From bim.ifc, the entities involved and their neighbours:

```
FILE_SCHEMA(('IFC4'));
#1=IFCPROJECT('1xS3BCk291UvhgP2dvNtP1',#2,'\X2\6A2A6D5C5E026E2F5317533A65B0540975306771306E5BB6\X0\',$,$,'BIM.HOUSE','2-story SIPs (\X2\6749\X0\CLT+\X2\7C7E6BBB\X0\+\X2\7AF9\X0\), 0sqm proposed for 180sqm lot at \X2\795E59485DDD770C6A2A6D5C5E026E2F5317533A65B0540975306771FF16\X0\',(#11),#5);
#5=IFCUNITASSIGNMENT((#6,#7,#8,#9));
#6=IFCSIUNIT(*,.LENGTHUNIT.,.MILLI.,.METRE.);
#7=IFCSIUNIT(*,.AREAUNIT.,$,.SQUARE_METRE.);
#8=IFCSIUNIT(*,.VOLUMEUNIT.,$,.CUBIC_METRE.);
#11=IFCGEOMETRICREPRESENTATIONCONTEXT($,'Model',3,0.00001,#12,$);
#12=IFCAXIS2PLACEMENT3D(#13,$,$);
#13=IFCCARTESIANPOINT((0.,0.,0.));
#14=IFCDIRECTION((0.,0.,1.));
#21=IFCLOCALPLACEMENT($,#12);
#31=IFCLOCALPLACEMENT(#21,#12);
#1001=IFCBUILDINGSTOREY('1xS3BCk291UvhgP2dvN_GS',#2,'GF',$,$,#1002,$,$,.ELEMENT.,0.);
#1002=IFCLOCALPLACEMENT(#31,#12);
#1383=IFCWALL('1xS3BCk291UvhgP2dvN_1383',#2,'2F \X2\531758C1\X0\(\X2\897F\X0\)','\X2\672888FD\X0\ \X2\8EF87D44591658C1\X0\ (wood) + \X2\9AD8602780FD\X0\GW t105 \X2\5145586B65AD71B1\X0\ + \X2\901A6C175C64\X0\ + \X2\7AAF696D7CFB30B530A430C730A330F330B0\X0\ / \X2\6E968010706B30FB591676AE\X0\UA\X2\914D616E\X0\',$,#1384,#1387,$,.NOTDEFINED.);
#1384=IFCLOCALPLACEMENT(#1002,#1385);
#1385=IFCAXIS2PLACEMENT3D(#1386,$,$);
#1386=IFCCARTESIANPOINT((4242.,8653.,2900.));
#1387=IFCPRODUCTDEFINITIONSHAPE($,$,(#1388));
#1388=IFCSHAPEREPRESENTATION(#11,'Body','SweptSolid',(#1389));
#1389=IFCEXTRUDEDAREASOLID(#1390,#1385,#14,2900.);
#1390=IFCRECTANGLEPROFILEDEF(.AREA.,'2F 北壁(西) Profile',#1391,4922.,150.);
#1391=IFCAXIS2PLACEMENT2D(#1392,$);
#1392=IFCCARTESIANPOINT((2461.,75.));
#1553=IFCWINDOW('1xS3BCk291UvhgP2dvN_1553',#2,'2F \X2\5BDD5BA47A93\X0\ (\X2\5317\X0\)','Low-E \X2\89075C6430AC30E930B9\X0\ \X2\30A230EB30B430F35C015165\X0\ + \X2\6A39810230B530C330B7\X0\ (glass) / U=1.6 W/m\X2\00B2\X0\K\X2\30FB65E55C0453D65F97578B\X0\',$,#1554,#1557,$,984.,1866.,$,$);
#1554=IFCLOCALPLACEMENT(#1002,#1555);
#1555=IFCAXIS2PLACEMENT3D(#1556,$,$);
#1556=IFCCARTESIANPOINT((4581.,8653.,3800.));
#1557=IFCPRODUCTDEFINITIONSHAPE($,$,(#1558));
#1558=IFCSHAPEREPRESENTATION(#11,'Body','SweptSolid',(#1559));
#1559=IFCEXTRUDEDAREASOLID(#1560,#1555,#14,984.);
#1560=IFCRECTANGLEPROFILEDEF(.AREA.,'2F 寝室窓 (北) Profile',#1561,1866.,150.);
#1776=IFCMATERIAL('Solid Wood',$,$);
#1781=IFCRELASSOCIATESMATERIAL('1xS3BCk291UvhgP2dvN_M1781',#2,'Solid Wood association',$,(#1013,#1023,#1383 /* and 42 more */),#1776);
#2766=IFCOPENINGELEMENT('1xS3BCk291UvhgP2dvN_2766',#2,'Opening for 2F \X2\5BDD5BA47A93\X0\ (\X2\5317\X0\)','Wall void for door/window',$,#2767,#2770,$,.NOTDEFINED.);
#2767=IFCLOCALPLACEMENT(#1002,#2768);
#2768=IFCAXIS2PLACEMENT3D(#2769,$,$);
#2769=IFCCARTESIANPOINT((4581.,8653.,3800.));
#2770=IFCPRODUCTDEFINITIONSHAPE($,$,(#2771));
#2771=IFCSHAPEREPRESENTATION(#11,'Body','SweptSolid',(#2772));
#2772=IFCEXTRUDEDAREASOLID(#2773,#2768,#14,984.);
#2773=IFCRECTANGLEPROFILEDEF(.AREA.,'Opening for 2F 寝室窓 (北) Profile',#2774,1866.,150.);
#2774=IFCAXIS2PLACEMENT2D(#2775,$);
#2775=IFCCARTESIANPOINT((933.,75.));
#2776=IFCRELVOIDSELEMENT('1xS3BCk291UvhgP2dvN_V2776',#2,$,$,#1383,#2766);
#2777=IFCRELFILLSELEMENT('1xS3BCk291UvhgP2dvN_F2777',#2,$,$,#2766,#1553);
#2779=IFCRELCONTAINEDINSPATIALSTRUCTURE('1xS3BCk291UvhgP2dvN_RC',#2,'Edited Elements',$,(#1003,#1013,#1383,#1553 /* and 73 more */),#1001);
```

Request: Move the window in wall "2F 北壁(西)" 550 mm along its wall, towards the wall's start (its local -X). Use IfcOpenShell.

```python
import ifcopenshell
import ifcopenshell.api.geometry
import ifcopenshell.util.placement

model = ifcopenshell.open("bim.ifc")

window = model.by_guid("1xS3BCk291UvhgP2dvN_1553")
opening = window.FillsVoids[0].RelatingOpeningElement
wall = opening.VoidsElements[0].RelatingBuildingElement

wall_matrix = ifcopenshell.util.placement.get_local_placement(wall.ObjectPlacement)
shift = wall_matrix[:3, 0] * -550.0
before = ifcopenshell.util.placement.get_local_placement(window.ObjectPlacement)[:3, 3].copy()

# The window is not placed relative to its opening, so move both.
for product in (opening, window):
    matrix = ifcopenshell.util.placement.get_local_placement(product.ObjectPlacement)
    matrix[:3, 3] += shift
    ifcopenshell.api.geometry.edit_object_placement(model, product=product, matrix=matrix, is_si=False)

after = ifcopenshell.util.placement.get_local_placement(window.ObjectPlacement)[:3, 3]
print("window moved by", (after - before).round(3) + 0.0)

model.write("bim_updated.ifc")
```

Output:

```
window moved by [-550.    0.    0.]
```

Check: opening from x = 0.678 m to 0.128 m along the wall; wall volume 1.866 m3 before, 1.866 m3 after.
